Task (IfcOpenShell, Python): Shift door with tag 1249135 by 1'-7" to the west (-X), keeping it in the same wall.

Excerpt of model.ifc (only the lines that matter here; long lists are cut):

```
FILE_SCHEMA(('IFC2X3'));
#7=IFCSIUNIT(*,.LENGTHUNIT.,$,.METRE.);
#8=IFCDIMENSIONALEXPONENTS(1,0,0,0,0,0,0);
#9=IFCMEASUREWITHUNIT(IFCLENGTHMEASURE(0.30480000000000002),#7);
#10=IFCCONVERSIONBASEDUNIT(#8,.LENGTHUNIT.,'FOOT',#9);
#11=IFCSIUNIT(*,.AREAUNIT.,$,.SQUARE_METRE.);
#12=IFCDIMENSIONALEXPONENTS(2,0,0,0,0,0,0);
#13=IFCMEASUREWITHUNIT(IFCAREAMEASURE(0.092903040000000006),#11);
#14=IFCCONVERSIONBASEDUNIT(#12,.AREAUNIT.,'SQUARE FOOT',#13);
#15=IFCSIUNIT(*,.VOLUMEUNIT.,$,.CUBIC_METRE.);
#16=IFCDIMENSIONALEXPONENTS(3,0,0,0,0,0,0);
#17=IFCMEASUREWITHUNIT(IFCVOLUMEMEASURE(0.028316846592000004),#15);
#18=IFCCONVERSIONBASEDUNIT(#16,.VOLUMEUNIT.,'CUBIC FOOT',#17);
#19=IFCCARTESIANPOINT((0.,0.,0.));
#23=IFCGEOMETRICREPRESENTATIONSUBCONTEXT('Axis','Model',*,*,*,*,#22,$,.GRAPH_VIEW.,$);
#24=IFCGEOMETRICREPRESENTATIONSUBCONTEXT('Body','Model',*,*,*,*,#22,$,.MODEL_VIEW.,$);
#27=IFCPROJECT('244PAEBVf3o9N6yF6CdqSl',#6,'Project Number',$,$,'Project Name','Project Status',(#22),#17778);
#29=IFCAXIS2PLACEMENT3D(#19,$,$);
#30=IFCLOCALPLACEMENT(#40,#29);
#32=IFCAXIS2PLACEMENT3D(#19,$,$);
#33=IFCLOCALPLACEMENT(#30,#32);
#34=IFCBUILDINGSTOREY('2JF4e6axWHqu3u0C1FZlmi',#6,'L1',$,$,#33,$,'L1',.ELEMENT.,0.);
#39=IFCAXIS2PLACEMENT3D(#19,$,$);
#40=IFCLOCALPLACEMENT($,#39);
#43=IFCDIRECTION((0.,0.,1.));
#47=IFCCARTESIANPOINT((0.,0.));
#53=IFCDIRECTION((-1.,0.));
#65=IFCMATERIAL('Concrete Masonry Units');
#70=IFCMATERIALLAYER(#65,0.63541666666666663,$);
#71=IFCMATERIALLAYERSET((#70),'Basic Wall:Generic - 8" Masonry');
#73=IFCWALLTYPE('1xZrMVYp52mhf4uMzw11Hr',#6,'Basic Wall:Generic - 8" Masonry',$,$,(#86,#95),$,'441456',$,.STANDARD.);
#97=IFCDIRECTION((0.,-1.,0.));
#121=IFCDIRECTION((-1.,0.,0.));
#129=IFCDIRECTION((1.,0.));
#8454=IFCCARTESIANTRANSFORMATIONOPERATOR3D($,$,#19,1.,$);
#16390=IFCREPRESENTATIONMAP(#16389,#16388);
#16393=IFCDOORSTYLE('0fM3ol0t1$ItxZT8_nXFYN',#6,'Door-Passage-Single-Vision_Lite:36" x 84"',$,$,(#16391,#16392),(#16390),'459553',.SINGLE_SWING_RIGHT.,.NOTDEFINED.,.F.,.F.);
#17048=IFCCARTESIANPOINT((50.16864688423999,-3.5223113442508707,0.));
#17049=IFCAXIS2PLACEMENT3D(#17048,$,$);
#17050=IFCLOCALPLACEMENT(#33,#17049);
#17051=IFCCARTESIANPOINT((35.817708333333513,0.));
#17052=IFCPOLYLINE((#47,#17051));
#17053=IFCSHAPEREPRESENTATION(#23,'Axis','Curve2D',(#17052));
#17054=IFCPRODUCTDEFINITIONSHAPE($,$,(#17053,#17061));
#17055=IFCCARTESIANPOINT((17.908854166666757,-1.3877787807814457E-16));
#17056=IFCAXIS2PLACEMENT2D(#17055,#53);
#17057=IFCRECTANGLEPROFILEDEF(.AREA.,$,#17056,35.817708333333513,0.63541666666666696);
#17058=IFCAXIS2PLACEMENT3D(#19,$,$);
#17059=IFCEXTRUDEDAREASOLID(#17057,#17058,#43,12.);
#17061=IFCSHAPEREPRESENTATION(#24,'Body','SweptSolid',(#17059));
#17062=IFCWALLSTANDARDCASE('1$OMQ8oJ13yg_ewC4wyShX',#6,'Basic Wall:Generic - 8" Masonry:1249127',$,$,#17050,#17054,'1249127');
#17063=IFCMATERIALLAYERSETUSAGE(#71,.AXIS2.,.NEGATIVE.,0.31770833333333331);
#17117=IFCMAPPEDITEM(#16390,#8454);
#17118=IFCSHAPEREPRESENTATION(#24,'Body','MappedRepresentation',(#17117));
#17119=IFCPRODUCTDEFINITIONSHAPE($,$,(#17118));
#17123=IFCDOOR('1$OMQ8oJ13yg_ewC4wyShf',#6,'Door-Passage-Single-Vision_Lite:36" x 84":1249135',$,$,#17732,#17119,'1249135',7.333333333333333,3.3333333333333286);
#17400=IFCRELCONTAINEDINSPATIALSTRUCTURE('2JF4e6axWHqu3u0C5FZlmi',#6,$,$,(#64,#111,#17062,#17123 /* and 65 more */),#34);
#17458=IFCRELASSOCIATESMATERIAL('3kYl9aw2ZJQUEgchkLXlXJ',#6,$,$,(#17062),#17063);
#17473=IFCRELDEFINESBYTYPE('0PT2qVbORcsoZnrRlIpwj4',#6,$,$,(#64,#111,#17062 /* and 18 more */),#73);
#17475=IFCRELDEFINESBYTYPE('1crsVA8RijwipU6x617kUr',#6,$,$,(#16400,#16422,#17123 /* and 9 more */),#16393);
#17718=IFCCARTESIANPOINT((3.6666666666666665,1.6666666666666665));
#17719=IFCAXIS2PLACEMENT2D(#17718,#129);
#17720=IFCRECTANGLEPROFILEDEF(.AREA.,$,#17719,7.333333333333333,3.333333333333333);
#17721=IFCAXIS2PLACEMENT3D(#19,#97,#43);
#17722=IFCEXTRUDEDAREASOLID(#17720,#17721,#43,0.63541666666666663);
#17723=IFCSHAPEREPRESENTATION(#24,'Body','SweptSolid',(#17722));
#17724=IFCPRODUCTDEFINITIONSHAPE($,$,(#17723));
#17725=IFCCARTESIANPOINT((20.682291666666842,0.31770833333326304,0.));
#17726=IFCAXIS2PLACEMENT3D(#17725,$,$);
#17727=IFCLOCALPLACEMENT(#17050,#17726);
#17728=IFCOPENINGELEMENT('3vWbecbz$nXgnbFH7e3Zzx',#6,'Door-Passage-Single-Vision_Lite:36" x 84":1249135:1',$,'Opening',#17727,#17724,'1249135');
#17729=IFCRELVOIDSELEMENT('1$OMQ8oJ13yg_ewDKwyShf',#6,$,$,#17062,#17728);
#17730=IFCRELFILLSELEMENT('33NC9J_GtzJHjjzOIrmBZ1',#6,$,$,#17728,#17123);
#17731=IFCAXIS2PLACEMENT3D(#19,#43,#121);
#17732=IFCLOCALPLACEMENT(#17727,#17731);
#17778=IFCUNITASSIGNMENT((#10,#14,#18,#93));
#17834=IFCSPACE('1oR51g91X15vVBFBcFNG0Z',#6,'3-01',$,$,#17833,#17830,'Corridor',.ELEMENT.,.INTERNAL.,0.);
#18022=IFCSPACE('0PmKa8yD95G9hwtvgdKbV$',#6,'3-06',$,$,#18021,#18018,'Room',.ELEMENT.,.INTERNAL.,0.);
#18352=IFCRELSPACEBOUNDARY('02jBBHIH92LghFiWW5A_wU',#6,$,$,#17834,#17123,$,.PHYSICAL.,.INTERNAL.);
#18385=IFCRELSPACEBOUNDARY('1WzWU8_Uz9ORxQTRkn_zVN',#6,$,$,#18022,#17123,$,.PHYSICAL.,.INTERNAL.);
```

```python
import ifcopenshell
import ifcopenshell.api.geometry
import ifcopenshell.util.placement
import ifcopenshell.util.unit

model = ifcopenshell.open("model.ifc")
unit_scale = ifcopenshell.util.unit.calculate_unit_scale(model)

door = model.by_guid("1$OMQ8oJ13yg_ewC4wyShf")
opening = door.FillsVoids[0].RelatingOpeningElement
wall = opening.VoidsElements[0].RelatingBuildingElement

wall_matrix = ifcopenshell.util.placement.get_local_placement(wall.ObjectPlacement)
shift = wall_matrix[:3, 0] * -19 * 0.0254 / unit_scale
before = ifcopenshell.util.placement.get_local_placement(door.ObjectPlacement)[:3, 3].copy()

# The door is placed relative to its opening, so it follows when the opening moves.
matrix = ifcopenshell.util.placement.get_local_placement(opening.ObjectPlacement)
matrix[:3, 3] += shift
ifcopenshell.api.geometry.edit_object_placement(
    model, product=opening, matrix=matrix, is_si=False, should_transform_children=True
)

after = ifcopenshell.util.placement.get_local_placement(door.ObjectPlacement)[:3, 3]
print("door moved by", (after - before).round(3) + 0.0)

model.write("model_rev.ifc")
```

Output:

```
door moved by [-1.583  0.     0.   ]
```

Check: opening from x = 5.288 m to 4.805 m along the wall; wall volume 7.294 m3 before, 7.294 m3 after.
